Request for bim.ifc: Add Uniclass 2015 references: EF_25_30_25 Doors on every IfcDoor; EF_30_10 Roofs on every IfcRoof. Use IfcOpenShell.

First a look at what the model holds.

```python
import ifcopenshell

model = ifcopenshell.open("bim.ifc")
print(model.schema)
print("classifications:", [c.Name for c in model.by_type("IfcClassification")])
for ifc_class in ("IfcDoor", "IfcRoof", "IfcStair", "IfcWall", "IfcWindow"):
    print(ifc_class, len(model.by_type(ifc_class)))
```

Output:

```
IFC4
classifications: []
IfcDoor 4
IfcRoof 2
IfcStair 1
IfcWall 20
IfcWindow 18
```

```python
import ifcopenshell
import ifcopenshell.api.classification

model = ifcopenshell.open("bim.ifc")

system = ifcopenshell.api.classification.add_classification(model, classification="Uniclass 2015")

codes = {
    "IfcDoor": ("EF_25_30_25", "Doors"),
    "IfcRoof": ("EF_30_10", "Roofs"),
}
for ifc_class, (code, name) in codes.items():
    products = model.by_type(ifc_class)
    ifcopenshell.api.classification.add_reference(
        model, products=products, classification=system, identification=code, name=name
    )
    print(code, len(products))

model.write("bim_v2.ifc")
```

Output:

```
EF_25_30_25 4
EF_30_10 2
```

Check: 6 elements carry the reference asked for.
